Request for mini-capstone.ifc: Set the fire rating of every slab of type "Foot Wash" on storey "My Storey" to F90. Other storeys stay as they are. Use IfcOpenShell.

First a look at what the model holds.

```python
import ifcopenshell
import ifcopenshell.util.element

model = ifcopenshell.open("mini-capstone.ifc")
print(model.schema)
storey = next(s for s in model.by_type("IfcBuildingStorey") if s.Name == "My Storey")
slabs = [e for e in ifcopenshell.util.element.get_decomposition(storey) if e.is_a("IfcSlab")]
seen = {}
for e in slabs:
    element_type = ifcopenshell.util.element.get_type(e)
    key = (element_type.Name if element_type != e and element_type else None, ifcopenshell.util.element.get_pset(e, "Pset_SlabCommon", "FireRating"))
    seen[key] = seen.get(key, 0) + 1
for (name, value), count in sorted(seen.items(), key=str):
    print(count, "x", name, "|", value)
```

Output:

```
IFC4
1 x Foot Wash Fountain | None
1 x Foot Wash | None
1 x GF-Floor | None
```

```python
import ifcopenshell
import ifcopenshell.api.pset
import ifcopenshell.util.element

model = ifcopenshell.open("mini-capstone.ifc")

storey = next(s for s in model.by_type("IfcBuildingStorey") if s.Name == "My Storey")
slabs = [e for e in ifcopenshell.util.element.get_decomposition(storey) if e.is_a("IfcSlab")]

count = 0
for e in slabs:
    element_type = ifcopenshell.util.element.get_type(e)
    if element_type in (None, e) or element_type.Name != "Foot Wash":
        continue
    # add_pset returns the element's existing set when there is one.
    pset = ifcopenshell.api.pset.add_pset(model, product=e, name="Pset_SlabCommon")
    ifcopenshell.api.pset.edit_pset(model, pset=pset, properties={"FireRating": "F90"})
    count += 1

print(count, "slabs updated")

model.write("mini-capstone_updated.ifc")
```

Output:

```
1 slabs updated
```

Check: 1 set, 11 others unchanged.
